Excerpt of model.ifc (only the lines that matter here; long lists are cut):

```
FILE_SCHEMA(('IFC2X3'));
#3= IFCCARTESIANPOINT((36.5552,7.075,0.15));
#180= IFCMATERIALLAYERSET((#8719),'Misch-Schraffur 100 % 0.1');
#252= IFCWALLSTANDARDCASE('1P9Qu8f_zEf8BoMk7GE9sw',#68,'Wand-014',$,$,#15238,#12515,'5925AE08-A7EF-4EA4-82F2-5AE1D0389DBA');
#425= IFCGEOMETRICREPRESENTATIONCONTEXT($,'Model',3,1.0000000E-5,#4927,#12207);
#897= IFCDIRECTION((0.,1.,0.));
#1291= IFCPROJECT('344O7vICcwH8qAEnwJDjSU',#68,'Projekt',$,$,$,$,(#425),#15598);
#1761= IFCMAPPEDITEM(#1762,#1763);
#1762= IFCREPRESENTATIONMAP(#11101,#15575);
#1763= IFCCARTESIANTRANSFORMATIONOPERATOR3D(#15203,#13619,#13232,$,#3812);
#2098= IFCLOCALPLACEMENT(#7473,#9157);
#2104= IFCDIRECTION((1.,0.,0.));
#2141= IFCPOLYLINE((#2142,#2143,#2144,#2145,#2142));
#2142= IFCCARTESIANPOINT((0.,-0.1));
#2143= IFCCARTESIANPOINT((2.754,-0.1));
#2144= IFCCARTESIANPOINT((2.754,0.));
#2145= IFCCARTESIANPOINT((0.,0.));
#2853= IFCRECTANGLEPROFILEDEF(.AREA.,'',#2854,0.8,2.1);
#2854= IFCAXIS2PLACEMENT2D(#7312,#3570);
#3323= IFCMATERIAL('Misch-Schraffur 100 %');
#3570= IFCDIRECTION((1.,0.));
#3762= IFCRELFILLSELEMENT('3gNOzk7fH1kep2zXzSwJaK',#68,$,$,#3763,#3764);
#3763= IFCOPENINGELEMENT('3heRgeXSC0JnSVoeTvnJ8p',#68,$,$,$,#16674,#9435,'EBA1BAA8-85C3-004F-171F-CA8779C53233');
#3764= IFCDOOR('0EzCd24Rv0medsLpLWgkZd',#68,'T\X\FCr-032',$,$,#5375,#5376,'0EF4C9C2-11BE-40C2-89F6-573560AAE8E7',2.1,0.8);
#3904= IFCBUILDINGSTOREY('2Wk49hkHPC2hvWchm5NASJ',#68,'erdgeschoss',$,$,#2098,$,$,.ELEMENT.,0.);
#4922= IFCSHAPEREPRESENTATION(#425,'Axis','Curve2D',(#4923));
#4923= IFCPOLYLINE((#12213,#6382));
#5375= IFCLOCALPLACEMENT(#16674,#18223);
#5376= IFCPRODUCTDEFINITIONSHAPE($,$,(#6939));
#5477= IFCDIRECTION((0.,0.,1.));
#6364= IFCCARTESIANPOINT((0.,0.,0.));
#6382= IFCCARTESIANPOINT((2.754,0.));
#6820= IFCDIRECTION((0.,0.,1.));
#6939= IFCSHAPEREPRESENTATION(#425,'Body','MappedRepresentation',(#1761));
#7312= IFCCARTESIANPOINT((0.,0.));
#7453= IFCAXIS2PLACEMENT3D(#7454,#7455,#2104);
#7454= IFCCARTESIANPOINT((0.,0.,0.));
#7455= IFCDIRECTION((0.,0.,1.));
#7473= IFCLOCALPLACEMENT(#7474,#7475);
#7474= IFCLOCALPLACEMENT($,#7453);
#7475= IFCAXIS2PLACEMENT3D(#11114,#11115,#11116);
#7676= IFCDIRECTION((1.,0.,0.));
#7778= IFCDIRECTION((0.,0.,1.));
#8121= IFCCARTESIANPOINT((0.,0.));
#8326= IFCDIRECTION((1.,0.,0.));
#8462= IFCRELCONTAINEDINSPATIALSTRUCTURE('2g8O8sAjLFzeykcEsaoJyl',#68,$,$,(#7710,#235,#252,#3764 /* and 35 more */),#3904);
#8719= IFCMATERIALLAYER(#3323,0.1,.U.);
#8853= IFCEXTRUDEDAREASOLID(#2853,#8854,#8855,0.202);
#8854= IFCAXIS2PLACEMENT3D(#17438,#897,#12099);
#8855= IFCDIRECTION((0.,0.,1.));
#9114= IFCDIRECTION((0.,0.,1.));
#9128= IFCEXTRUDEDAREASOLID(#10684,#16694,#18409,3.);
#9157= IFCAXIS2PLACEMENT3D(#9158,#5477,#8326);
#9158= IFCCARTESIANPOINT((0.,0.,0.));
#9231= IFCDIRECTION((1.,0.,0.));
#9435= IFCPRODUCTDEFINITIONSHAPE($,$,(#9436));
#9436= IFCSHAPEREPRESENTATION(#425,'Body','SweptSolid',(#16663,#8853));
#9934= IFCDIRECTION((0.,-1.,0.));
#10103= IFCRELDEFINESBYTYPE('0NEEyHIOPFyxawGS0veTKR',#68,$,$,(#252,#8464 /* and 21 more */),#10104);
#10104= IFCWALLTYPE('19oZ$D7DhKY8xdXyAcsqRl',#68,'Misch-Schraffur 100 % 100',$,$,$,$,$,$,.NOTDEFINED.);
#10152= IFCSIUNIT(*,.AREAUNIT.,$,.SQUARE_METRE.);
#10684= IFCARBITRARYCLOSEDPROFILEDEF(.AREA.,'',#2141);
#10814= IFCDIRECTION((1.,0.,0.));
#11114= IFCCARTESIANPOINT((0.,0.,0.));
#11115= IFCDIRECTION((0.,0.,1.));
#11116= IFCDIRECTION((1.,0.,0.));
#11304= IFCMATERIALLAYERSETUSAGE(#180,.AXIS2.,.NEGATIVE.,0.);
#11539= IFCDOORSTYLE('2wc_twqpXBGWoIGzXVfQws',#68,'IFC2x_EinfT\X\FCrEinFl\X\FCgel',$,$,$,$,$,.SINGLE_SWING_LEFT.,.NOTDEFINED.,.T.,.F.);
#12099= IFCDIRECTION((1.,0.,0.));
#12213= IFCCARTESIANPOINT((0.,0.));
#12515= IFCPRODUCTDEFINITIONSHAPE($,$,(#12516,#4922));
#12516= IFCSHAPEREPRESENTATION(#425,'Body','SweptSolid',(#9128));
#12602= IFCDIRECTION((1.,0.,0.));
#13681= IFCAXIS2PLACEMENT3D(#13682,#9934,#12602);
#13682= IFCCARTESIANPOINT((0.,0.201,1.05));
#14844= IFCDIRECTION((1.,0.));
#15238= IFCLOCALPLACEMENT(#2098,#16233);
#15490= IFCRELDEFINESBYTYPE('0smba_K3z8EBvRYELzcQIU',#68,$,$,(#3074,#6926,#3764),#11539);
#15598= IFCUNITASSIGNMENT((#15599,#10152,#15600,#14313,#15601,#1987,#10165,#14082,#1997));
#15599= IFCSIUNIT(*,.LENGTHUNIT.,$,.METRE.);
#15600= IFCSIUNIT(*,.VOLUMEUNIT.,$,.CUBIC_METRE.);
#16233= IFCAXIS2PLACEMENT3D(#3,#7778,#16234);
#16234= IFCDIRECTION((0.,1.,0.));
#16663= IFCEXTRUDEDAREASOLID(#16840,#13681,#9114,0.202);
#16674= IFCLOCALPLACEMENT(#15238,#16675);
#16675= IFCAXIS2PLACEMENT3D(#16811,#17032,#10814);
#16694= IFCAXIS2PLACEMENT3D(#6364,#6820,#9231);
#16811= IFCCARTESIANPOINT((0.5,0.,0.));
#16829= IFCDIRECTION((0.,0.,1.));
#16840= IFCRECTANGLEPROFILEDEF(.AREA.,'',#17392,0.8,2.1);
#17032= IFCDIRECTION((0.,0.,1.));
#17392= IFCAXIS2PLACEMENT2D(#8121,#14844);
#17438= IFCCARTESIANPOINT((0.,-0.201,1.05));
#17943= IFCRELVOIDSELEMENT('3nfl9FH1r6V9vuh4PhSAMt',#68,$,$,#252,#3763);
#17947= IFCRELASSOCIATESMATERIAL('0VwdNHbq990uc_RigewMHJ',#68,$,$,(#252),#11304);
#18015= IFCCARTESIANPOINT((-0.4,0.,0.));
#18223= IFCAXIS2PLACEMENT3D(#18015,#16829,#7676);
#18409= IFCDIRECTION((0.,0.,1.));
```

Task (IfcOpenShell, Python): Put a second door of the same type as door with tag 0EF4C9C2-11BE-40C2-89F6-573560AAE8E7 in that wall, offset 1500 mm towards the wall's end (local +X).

```python
import ifcopenshell
import ifcopenshell.api.feature
import ifcopenshell.api.geometry
import ifcopenshell.api.root
import ifcopenshell.geom
import ifcopenshell.util.element
import ifcopenshell.util.placement
import ifcopenshell.util.shape

model = ifcopenshell.open("model.ifc")
settings = ifcopenshell.geom.settings()


def volume(element):
    """Net volume in cubic metres, openings subtracted."""
    shape = ifcopenshell.geom.create_shape(settings, element)
    return ifcopenshell.util.shape.get_volume(shape.geometry)


def reuse_history(source, copy):
    """copy_class also copies each property set's owner history, people and application; keep the originals."""
    for rel in copy.IsDefinedBy:
        if rel.is_a("IfcRelDefinesByProperties") and (history := rel.RelatingPropertyDefinition.OwnerHistory):
            rel.RelatingPropertyDefinition.OwnerHistory = source.OwnerHistory
            ifcopenshell.util.element.remove_deep2(model, history)


door = model.by_guid("0EzCd24Rv0medsLpLWgkZd")
opening = door.FillsVoids[0].RelatingOpeningElement
wall = opening.VoidsElements[0].RelatingBuildingElement
before = volume(wall)
shift = ifcopenshell.util.placement.get_local_placement(wall.ObjectPlacement)[:3, 0] * 1.5

# copy_class copies the void relationship, type, container and properties, but no geometry.
new_opening = ifcopenshell.api.root.copy_class(model, product=opening)
new_opening.Representation = ifcopenshell.util.element.copy_deep(
    model, opening.Representation, exclude=["IfcGeometricRepresentationContext", "IfcRepresentationMap"]
)
new_opening.Tag = None
new_door = ifcopenshell.api.root.copy_class(model, product=door)
new_door.Representation = ifcopenshell.util.element.copy_deep(
    model, door.Representation, exclude=["IfcGeometricRepresentationContext", "IfcRepresentationMap"]
)
new_door.Tag = None
reuse_history(door, new_door)
fills = ifcopenshell.api.feature.add_filling(model, opening=new_opening, element=new_door)
fills.OwnerHistory = new_door.OwnerHistory  # required in IFC2X3

for old, new in ((opening, new_opening), (door, new_door)):
    matrix = ifcopenshell.util.placement.get_local_placement(old.ObjectPlacement)
    matrix[:3, 3] += shift
    ifcopenshell.api.geometry.edit_object_placement(model, product=new, matrix=matrix, is_si=False)

after = volume(wall)

print(f"wall volume {before:.3f} -> {after:.3f} m3")

model.write("model-out.ifc")
```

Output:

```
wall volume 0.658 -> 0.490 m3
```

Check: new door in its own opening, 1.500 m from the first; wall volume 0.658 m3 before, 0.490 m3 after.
